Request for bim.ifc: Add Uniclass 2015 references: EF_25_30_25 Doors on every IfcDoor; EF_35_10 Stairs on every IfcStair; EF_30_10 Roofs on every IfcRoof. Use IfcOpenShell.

First a look at what the model holds.

```python
import ifcopenshell

model = ifcopenshell.open("bim.ifc")
print(model.schema)
print("classifications:", [c.Name for c in model.by_type("IfcClassification")])
for ifc_class in ("IfcDoor", "IfcRoof", "IfcStair", "IfcWall", "IfcWindow"):
    print(ifc_class, len(model.by_type(ifc_class)))
```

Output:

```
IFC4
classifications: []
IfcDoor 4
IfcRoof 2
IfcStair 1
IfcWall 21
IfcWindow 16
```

```python
import ifcopenshell
import ifcopenshell.api.classification

model = ifcopenshell.open("bim.ifc")

system = ifcopenshell.api.classification.add_classification(model, classification="Uniclass 2015")

codes = {
    "IfcDoor": ("EF_25_30_25", "Doors"),
    "IfcStair": ("EF_35_10", "Stairs"),
    "IfcRoof": ("EF_30_10", "Roofs"),
}
for ifc_class, (code, name) in codes.items():
    products = model.by_type(ifc_class)
    ifcopenshell.api.classification.add_reference(
        model, products=products, classification=system, identification=code, name=name
    )
    print(code, len(products))

model.write("bim-out.ifc")
```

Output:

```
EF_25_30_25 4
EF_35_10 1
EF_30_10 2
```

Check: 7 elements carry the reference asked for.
